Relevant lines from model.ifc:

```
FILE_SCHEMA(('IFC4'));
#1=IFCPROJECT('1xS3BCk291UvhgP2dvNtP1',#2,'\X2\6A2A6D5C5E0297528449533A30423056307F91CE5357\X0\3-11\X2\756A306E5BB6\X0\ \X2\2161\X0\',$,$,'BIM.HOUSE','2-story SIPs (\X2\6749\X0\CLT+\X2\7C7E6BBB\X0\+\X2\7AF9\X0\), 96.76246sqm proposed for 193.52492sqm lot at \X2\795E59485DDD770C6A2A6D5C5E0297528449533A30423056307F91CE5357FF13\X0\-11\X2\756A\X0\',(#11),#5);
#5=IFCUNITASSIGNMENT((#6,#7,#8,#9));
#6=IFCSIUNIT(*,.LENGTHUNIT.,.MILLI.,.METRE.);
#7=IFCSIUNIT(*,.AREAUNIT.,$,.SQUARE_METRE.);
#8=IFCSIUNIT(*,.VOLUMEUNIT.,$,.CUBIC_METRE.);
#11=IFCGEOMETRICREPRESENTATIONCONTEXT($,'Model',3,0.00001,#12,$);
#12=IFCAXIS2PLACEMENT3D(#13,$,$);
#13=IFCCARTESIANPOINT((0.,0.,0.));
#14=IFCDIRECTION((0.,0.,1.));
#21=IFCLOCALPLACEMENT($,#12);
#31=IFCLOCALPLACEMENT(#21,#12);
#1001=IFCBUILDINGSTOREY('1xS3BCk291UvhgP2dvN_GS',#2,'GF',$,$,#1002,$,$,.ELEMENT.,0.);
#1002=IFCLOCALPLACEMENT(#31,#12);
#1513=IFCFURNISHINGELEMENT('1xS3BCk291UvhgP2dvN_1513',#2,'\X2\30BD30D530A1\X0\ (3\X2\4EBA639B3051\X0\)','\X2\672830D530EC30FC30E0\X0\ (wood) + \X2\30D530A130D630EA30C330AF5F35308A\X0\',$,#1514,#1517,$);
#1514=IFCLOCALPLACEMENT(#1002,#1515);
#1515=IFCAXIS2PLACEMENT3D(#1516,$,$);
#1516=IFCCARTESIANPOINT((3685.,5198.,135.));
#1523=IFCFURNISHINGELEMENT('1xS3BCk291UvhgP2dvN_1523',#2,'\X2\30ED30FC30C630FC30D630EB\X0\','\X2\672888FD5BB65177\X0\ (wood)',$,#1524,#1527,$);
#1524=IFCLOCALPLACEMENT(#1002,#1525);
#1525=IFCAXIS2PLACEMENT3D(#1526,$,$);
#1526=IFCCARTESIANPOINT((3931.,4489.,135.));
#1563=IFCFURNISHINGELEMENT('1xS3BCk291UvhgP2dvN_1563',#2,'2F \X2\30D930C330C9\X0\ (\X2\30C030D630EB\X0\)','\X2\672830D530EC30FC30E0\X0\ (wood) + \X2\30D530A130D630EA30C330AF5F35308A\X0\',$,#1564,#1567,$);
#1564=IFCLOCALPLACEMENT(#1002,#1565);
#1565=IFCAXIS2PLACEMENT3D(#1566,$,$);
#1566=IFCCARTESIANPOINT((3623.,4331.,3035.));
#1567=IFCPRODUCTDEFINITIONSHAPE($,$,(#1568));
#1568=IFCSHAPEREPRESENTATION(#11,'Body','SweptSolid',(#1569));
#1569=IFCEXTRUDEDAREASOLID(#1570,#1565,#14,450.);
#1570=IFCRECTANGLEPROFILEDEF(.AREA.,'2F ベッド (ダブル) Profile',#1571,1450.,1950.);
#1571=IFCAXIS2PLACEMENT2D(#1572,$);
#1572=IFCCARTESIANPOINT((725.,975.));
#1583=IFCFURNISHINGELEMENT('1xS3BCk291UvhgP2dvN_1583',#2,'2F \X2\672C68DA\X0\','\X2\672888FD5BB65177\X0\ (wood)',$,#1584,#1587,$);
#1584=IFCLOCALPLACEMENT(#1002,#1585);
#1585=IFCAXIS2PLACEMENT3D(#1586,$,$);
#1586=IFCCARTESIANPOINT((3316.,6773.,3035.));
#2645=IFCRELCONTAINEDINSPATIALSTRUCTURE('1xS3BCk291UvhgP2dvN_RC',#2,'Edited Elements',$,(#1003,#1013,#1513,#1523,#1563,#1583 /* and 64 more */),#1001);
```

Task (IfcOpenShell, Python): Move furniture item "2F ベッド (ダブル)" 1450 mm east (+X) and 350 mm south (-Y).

```python
import ifcopenshell
import ifcopenshell.api.geometry
import ifcopenshell.util.placement
import ifcopenshell.util.unit

model = ifcopenshell.open("model.ifc")
unit_scale = ifcopenshell.util.unit.calculate_unit_scale(model)

item = model.by_guid("1xS3BCk291UvhgP2dvN_1563")
matrix = ifcopenshell.util.placement.get_local_placement(item.ObjectPlacement)
matrix[0, 3] += 1.45 / unit_scale
matrix[1, 3] -= 0.35 / unit_scale
ifcopenshell.api.geometry.edit_object_placement(model, product=item, matrix=matrix, is_si=False)

print(ifcopenshell.util.placement.get_local_placement(item.ObjectPlacement).round(3) + 0.0)

model.write("model-out.ifc")
```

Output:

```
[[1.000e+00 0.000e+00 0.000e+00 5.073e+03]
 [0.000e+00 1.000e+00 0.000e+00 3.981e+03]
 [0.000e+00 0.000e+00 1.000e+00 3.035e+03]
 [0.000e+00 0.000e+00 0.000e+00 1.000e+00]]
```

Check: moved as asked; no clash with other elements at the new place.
